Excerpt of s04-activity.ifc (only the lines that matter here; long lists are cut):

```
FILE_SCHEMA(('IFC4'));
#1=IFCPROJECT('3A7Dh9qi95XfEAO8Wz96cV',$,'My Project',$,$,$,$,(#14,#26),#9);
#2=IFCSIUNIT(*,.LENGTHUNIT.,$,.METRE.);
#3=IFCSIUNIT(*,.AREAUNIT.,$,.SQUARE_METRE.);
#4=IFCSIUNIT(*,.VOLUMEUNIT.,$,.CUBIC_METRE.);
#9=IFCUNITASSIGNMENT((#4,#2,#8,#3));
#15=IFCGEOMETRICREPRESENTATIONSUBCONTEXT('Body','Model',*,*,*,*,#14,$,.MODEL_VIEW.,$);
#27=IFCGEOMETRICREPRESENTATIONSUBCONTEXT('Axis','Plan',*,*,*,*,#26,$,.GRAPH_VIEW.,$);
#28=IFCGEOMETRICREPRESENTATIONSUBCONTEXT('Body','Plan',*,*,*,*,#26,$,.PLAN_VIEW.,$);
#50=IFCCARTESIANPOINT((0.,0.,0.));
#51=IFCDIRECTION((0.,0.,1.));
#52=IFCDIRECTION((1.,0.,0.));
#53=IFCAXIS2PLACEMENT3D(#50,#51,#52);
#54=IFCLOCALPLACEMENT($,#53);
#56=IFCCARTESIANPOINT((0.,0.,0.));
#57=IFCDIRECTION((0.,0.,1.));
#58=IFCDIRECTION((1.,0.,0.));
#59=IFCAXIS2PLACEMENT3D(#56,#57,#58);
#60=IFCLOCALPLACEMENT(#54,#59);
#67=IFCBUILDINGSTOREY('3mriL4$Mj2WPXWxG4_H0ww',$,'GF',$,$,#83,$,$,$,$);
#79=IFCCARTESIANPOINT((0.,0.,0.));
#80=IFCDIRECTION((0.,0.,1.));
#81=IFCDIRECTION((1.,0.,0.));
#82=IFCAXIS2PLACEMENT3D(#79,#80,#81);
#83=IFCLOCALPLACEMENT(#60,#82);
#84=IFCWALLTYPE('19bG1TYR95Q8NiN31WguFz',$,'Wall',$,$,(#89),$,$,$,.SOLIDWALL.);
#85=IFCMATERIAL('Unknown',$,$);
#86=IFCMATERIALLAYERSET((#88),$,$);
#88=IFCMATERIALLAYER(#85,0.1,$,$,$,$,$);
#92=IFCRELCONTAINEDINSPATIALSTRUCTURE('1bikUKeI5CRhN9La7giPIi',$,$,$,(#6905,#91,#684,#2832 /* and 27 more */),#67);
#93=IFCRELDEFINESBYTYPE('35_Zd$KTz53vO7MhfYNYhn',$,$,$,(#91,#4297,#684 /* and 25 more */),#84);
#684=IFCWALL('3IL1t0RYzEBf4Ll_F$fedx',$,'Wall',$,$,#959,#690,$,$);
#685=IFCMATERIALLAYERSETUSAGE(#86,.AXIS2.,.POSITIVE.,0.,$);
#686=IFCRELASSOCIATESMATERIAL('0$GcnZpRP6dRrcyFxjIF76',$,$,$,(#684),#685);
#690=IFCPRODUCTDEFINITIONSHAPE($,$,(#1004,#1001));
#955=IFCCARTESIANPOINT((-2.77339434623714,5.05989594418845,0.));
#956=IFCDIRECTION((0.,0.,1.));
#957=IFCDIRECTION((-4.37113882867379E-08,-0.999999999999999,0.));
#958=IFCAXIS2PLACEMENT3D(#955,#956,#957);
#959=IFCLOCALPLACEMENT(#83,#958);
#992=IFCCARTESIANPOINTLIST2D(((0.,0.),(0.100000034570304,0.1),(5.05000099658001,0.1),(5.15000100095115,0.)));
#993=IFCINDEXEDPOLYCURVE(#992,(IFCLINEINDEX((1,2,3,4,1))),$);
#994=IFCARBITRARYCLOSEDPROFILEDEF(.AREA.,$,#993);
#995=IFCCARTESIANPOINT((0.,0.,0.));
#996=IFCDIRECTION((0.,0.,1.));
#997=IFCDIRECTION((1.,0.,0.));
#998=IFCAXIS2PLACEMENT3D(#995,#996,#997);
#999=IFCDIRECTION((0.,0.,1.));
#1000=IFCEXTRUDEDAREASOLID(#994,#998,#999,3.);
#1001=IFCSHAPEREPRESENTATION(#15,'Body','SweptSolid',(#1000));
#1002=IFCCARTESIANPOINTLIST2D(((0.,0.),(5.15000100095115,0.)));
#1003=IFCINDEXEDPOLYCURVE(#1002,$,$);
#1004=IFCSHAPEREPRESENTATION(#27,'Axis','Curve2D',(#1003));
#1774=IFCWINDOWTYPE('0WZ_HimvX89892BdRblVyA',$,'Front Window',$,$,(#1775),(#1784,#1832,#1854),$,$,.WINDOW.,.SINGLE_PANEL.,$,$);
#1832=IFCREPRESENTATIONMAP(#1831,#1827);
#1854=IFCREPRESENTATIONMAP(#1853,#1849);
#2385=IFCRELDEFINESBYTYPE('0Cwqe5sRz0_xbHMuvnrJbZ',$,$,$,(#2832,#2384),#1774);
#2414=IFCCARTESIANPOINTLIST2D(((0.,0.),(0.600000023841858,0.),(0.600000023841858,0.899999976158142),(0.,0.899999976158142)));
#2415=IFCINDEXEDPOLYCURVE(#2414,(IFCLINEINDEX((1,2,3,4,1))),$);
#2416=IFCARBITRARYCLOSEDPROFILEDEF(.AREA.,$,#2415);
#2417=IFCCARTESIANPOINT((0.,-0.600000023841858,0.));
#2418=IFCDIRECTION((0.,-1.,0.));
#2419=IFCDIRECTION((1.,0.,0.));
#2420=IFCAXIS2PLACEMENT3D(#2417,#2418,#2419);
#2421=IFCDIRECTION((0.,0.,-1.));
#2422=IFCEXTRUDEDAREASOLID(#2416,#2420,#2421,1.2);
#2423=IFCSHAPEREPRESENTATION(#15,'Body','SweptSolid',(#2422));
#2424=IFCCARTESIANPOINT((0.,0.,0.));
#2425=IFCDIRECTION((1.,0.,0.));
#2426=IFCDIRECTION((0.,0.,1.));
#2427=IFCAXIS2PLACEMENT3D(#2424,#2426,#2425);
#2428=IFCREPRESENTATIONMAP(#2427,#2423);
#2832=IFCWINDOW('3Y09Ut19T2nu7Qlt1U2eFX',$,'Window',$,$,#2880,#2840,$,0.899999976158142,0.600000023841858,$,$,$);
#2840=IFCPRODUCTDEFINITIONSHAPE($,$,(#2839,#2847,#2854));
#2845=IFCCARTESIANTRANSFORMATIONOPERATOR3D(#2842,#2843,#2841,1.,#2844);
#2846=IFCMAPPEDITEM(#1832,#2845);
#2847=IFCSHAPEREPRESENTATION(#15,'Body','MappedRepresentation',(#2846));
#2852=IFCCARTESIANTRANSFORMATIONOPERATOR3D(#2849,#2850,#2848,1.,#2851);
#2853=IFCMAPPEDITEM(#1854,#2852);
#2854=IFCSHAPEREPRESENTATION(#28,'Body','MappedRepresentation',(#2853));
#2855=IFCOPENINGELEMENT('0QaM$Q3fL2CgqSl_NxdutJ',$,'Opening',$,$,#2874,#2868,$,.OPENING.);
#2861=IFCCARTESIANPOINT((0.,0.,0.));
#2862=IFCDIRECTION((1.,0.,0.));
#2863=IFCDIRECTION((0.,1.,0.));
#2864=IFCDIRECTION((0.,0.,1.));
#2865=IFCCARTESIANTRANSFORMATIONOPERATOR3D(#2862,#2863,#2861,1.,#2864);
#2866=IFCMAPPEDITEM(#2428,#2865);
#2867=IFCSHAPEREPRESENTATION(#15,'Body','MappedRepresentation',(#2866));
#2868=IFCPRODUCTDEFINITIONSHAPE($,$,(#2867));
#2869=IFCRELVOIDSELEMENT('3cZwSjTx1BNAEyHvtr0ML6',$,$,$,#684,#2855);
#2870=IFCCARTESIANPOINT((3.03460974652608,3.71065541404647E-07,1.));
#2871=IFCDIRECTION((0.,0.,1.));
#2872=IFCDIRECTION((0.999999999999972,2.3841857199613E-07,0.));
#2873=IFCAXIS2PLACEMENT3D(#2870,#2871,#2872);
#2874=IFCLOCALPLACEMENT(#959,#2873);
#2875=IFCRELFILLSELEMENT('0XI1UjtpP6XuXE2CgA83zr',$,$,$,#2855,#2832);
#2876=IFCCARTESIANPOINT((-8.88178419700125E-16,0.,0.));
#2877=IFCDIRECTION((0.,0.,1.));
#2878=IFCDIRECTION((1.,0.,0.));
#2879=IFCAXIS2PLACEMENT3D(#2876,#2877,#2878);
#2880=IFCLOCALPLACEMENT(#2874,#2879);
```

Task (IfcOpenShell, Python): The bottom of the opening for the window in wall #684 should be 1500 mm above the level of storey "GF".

```python
import numpy as np
import ifcopenshell
import ifcopenshell.api.geometry
import ifcopenshell.geom
import ifcopenshell.util.element
import ifcopenshell.util.placement
import ifcopenshell.util.shape
import ifcopenshell.util.unit

model = ifcopenshell.open("s04-activity.ifc")
unit_scale = ifcopenshell.util.unit.calculate_unit_scale(model)

window = model.by_id(2832)
opening = window.FillsVoids[0].RelatingOpeningElement
storey = ifcopenshell.util.element.get_container(window, ifc_class="IfcBuildingStorey")
level = ifcopenshell.util.placement.get_local_placement(storey.ObjectPlacement)[2, 3]

# The opening's origin need not be at the sill, so measure its lowest point.
shape = ifcopenshell.geom.create_shape(ifcopenshell.geom.settings(), opening)
bottom = ifcopenshell.util.shape.get_shape_bottom_elevation(shape, shape.geometry) / unit_scale
dz = level + 1.5 / unit_scale - bottom

shift = np.array([0.0, 0.0, dz])
# The window is placed relative to its opening, so it follows when the opening moves.
matrix = ifcopenshell.util.placement.get_local_placement(opening.ObjectPlacement)
matrix[:3, 3] += shift
ifcopenshell.api.geometry.edit_object_placement(
    model, product=opening, matrix=matrix, is_si=False, should_transform_children=True
)

print(f"moved by {dz * unit_scale:+.3f} m")

model.write("s04-activity_updated.ifc")
```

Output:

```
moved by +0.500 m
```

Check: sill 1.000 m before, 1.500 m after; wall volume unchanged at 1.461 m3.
